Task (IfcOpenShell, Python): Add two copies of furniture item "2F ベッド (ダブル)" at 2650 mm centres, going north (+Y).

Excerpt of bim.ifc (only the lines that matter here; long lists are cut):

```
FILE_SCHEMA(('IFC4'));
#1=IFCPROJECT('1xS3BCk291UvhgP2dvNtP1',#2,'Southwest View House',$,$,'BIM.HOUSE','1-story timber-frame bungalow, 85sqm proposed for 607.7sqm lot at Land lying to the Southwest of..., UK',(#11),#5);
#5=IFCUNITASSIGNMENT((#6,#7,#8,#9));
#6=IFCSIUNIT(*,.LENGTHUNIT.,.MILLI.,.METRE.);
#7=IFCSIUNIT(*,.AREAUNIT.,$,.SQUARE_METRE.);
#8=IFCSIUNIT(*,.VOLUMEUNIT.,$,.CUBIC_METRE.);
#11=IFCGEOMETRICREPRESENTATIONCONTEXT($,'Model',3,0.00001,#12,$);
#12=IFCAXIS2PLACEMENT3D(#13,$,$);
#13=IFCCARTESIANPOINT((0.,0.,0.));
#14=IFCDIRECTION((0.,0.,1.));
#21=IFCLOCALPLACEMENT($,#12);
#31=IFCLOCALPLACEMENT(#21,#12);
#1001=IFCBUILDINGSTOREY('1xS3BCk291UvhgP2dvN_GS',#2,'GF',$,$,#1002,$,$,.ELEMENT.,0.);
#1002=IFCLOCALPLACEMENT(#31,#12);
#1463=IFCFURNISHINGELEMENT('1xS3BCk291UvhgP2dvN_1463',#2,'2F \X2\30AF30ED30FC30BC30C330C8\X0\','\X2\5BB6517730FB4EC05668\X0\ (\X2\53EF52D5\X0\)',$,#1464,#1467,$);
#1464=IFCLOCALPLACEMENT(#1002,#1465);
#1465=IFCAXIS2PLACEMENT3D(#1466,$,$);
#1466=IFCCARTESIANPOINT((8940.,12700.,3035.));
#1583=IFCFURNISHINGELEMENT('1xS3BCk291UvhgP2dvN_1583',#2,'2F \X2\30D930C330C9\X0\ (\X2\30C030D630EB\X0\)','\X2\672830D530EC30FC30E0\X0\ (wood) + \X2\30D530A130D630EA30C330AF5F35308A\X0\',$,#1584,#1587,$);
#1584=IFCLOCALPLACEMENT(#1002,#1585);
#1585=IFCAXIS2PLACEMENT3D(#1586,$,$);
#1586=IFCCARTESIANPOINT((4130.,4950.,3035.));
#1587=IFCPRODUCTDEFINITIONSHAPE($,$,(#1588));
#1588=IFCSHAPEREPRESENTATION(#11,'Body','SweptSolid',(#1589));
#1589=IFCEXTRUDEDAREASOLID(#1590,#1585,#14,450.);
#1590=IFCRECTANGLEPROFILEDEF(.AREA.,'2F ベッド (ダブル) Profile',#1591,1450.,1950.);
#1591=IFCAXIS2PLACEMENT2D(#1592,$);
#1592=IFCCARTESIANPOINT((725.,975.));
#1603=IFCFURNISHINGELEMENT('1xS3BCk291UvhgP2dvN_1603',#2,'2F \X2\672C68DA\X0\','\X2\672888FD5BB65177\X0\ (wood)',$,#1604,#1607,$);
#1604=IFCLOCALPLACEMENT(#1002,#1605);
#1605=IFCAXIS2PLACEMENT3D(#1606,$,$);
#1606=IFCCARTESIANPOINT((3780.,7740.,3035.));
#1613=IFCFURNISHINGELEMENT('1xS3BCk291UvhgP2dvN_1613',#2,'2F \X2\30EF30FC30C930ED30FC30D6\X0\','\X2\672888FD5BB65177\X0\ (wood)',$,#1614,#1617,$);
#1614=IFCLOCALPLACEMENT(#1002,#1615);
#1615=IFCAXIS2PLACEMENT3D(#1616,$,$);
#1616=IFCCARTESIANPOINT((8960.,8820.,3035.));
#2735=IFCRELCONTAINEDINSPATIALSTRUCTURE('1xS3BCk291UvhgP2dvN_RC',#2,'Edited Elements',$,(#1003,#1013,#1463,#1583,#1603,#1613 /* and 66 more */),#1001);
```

```python
import numpy as np
import ifcopenshell
import ifcopenshell.api.geometry
import ifcopenshell.api.root
import ifcopenshell.util.element
import ifcopenshell.util.placement
import ifcopenshell.util.unit

model = ifcopenshell.open("bim.ifc")
unit_scale = ifcopenshell.util.unit.calculate_unit_scale(model)


def reuse_history(source, copy):
    """copy_class also copies each property set's owner history, people and application; keep the originals."""
    for rel in copy.IsDefinedBy:
        if rel.is_a("IfcRelDefinesByProperties") and (history := rel.RelatingPropertyDefinition.OwnerHistory):
            rel.RelatingPropertyDefinition.OwnerHistory = source.OwnerHistory
            ifcopenshell.util.element.remove_deep2(model, history)


source = model.by_guid("1xS3BCk291UvhgP2dvN_1583")
base = ifcopenshell.util.placement.get_local_placement(source.ObjectPlacement)
step = np.array([0.0, 1.0, 0.0]) * 2.65 / unit_scale

for i in range(1, 3):
    copy = ifcopenshell.api.root.copy_class(model, product=source)
    copy.Representation = ifcopenshell.util.element.copy_deep(
        model, source.Representation, exclude=["IfcGeometricRepresentationContext", "IfcRepresentationMap"]
    )
    reuse_history(source, copy)
    matrix = base.copy()
    matrix[:3, 3] += i * step
    print("added at", matrix[:3, 3].round(3) + 0.0)
    ifcopenshell.api.geometry.edit_object_placement(model, product=copy, matrix=matrix, is_si=False)

model.write("bim_updated.ifc")
```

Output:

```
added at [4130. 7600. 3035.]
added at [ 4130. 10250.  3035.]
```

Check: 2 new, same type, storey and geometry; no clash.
